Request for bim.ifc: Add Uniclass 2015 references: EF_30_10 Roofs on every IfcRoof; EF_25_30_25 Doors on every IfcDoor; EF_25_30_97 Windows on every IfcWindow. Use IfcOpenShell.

First a look at what the model holds.

```python
import ifcopenshell

model = ifcopenshell.open("bim.ifc")
print(model.schema)
print("classifications:", [c.Name for c in model.by_type("IfcClassification")])
for ifc_class in ("IfcDoor", "IfcRoof", "IfcStair", "IfcWall", "IfcWindow"):
    print(ifc_class, len(model.by_type(ifc_class)))
```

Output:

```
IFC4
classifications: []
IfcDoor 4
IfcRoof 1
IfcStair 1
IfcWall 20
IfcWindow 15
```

```python
import ifcopenshell
import ifcopenshell.api.classification

model = ifcopenshell.open("bim.ifc")

system = ifcopenshell.api.classification.add_classification(model, classification="Uniclass 2015")

codes = {
    "IfcRoof": ("EF_30_10", "Roofs"),
    "IfcDoor": ("EF_25_30_25", "Doors"),
    "IfcWindow": ("EF_25_30_97", "Windows"),
}
for ifc_class, (code, name) in codes.items():
    products = model.by_type(ifc_class)
    ifcopenshell.api.classification.add_reference(
        model, products=products, classification=system, identification=code, name=name
    )
    print(code, len(products))

model.write("bim_rev.ifc")
```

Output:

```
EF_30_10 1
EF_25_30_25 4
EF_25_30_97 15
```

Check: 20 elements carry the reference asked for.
